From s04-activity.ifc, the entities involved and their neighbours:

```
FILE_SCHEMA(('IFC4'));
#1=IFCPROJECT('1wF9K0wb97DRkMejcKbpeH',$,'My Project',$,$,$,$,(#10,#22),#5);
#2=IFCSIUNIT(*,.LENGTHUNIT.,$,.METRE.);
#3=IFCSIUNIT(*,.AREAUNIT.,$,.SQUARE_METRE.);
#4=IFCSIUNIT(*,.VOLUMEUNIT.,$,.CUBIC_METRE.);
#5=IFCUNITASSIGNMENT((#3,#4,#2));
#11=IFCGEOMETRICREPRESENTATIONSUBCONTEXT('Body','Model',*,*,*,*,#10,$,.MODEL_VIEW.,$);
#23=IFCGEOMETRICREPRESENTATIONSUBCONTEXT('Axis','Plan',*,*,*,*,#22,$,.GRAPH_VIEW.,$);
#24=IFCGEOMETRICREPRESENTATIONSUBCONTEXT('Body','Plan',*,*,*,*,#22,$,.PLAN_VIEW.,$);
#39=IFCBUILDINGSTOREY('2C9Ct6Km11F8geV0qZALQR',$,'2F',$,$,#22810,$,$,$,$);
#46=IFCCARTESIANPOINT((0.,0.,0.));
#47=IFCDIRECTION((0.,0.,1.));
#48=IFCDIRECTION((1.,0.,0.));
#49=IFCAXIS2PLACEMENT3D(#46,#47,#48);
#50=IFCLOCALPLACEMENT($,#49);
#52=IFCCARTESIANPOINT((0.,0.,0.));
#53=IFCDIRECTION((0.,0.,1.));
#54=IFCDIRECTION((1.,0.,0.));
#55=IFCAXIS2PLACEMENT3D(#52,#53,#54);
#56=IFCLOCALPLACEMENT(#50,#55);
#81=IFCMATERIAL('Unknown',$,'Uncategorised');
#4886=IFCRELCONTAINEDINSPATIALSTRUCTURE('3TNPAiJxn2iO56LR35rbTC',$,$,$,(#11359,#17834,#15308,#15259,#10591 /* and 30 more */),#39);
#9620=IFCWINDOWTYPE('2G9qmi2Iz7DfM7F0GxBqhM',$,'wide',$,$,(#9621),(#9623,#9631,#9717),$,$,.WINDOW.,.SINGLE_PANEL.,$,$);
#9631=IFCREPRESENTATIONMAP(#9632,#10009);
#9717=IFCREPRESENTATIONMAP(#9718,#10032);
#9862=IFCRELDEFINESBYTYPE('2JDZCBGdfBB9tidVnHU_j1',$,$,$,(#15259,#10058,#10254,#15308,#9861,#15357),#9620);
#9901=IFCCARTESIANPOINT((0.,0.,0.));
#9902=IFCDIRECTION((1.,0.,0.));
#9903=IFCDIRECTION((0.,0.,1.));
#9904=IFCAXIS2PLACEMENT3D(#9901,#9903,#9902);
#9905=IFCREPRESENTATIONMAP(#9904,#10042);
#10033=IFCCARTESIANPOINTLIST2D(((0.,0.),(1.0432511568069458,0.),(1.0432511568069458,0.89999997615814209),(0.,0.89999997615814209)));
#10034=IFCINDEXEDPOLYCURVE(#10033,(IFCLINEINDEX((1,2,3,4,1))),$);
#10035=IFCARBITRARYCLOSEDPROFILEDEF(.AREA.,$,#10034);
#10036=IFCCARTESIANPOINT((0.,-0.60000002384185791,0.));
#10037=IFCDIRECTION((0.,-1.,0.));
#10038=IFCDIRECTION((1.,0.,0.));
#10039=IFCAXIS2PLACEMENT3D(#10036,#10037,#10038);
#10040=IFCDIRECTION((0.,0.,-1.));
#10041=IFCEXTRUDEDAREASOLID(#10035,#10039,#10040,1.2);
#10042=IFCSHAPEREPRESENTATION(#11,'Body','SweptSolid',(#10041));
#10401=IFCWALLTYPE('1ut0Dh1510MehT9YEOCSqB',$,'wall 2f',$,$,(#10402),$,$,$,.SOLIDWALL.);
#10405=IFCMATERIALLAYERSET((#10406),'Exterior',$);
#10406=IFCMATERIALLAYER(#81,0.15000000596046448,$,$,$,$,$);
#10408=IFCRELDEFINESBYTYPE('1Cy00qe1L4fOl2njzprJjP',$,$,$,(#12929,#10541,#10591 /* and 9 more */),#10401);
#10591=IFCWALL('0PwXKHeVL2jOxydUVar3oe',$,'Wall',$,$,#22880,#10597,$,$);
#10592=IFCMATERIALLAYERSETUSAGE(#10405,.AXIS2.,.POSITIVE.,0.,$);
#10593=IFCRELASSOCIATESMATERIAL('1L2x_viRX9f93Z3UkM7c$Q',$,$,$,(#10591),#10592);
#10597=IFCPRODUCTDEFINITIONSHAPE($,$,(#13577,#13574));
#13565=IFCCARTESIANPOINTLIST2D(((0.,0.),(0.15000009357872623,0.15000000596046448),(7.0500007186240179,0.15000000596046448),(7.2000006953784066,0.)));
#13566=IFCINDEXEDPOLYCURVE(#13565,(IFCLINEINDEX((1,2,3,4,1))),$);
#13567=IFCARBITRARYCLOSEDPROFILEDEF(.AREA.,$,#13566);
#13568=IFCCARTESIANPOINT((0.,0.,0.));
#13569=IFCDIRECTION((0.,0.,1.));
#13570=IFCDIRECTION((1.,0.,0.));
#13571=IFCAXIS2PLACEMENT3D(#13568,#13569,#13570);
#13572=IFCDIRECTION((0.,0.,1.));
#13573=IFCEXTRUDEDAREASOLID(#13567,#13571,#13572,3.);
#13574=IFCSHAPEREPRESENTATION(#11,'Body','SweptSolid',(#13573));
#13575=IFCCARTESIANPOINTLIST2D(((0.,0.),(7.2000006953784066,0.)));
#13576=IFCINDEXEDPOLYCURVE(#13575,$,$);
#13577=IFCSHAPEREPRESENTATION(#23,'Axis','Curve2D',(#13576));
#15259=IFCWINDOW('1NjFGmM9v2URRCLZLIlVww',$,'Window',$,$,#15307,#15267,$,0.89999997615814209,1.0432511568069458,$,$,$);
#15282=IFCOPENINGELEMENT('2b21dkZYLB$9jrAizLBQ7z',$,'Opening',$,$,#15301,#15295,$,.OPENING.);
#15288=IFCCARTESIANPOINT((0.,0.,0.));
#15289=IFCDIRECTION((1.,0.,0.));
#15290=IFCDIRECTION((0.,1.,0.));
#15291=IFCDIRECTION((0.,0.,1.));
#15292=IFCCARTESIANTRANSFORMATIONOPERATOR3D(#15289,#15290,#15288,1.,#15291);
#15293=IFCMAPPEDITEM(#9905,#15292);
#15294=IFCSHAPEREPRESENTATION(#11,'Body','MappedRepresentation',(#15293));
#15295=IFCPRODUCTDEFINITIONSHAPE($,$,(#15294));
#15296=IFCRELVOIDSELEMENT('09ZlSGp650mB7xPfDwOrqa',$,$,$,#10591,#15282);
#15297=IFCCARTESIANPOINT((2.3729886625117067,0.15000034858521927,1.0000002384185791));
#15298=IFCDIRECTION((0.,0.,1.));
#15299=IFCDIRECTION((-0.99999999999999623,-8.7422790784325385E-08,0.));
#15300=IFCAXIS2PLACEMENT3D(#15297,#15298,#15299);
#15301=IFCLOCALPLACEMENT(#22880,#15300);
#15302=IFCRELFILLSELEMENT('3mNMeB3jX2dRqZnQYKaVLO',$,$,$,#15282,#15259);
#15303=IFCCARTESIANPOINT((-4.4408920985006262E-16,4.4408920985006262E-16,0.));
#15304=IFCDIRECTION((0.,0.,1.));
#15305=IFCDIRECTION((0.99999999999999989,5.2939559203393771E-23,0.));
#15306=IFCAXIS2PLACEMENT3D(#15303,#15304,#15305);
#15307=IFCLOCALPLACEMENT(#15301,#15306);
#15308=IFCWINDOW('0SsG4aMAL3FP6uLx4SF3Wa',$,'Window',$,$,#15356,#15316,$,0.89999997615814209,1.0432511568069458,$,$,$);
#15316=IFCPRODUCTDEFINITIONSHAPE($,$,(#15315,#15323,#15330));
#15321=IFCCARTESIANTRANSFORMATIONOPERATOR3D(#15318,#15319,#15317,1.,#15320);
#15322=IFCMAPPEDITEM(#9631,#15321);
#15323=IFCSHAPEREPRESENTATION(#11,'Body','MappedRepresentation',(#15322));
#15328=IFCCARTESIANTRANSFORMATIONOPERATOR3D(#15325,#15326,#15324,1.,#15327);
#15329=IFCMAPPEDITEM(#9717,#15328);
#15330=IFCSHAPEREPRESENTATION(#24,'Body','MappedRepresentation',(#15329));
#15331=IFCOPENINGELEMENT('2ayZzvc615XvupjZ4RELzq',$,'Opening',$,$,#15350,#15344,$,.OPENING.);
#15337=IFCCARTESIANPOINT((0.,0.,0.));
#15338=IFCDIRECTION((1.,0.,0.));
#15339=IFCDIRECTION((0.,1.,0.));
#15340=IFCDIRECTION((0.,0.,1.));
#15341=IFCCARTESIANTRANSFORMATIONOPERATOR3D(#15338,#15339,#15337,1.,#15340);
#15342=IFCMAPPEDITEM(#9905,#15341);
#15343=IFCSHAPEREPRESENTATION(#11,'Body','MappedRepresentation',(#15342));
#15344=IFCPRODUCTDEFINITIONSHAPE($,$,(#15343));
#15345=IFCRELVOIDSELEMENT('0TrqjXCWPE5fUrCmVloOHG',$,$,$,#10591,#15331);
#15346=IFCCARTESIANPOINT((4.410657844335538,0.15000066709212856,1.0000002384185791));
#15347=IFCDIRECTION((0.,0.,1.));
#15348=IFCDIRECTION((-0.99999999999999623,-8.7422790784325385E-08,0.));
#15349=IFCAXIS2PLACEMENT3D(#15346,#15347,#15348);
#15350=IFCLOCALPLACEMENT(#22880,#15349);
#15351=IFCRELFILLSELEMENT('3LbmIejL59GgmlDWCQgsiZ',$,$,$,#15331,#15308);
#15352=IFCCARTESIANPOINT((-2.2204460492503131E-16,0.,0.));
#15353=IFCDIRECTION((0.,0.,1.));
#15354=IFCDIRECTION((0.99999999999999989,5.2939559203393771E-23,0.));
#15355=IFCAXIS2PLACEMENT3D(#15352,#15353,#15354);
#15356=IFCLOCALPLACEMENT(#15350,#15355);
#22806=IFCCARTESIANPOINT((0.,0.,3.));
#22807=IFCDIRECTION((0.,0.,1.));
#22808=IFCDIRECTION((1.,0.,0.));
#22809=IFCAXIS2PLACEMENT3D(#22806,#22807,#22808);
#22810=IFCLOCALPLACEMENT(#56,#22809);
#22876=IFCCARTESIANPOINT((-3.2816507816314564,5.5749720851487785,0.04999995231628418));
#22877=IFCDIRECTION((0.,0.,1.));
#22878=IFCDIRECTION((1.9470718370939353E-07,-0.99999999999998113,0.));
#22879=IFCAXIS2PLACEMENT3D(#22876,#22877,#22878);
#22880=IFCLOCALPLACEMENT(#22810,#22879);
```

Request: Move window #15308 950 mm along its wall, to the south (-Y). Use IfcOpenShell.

```python
import ifcopenshell
import ifcopenshell.api.geometry
import ifcopenshell.util.placement

model = ifcopenshell.open("s04-activity.ifc")

window = model.by_id(15308)
opening = window.FillsVoids[0].RelatingOpeningElement
wall = opening.VoidsElements[0].RelatingBuildingElement

wall_matrix = ifcopenshell.util.placement.get_local_placement(wall.ObjectPlacement)
shift = wall_matrix[:3, 0] * 0.95
before = ifcopenshell.util.placement.get_local_placement(window.ObjectPlacement)[:3, 3].copy()

# The window is placed relative to its opening, so it follows when the opening moves.
matrix = ifcopenshell.util.placement.get_local_placement(opening.ObjectPlacement)
matrix[:3, 3] += shift
ifcopenshell.api.geometry.edit_object_placement(
    model, product=opening, matrix=matrix, is_si=False, should_transform_children=True
)

after = ifcopenshell.util.placement.get_local_placement(window.ObjectPlacement)[:3, 3]
print("window moved by", (after - before).round(3) + 0.0)

model.write("s04-activity_rev.ifc")
```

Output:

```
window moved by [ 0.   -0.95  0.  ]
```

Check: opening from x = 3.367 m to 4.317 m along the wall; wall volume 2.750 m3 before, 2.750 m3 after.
